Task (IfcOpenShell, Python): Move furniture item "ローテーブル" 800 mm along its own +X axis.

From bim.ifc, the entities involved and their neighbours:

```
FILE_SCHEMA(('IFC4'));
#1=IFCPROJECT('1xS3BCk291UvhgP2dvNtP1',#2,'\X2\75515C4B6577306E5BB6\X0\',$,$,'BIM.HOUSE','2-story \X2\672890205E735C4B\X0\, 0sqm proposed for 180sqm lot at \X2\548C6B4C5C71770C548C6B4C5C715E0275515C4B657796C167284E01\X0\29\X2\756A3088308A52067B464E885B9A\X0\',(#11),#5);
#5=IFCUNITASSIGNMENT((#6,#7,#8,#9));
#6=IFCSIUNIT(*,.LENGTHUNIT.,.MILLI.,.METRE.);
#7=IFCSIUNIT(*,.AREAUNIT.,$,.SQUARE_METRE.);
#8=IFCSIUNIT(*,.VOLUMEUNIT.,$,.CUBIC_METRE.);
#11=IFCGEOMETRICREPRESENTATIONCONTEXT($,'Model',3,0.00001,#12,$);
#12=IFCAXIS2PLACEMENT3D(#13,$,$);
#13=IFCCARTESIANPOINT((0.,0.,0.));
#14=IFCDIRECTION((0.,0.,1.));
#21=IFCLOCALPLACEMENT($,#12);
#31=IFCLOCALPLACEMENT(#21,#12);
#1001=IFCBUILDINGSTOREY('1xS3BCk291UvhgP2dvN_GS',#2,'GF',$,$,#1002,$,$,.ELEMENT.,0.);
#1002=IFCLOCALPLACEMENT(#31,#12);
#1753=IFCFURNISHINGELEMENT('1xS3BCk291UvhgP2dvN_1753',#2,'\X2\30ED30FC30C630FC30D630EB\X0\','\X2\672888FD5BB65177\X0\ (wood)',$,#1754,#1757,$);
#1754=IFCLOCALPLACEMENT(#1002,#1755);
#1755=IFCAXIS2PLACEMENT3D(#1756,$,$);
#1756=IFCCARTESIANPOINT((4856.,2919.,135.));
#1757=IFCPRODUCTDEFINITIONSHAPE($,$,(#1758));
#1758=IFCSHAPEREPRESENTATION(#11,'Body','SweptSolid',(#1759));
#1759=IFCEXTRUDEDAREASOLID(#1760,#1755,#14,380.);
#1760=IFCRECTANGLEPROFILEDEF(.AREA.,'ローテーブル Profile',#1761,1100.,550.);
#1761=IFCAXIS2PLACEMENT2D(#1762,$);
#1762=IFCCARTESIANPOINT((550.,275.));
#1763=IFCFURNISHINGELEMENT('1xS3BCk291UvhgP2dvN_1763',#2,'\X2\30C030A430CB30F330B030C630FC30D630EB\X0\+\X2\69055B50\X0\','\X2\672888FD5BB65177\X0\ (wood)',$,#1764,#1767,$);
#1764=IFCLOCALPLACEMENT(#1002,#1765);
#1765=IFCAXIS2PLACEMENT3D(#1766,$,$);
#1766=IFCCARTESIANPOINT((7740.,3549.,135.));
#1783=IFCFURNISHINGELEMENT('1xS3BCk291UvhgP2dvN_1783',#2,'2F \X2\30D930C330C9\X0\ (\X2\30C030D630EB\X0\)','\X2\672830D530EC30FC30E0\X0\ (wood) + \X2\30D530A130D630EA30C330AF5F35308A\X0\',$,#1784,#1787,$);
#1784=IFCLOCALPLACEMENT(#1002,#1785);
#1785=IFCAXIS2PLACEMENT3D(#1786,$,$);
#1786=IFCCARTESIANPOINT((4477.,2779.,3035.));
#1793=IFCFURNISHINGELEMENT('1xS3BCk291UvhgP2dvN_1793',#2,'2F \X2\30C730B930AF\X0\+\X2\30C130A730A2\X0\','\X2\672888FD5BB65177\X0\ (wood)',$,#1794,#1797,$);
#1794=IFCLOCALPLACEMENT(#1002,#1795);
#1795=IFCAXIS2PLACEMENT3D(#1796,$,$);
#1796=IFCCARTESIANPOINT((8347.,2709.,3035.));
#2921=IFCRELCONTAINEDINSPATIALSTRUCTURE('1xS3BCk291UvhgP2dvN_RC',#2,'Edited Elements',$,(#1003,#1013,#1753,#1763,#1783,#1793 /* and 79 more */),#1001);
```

```python
import ifcopenshell
import ifcopenshell.api.geometry
import ifcopenshell.util.placement
import ifcopenshell.util.unit

model = ifcopenshell.open("bim.ifc")
unit_scale = ifcopenshell.util.unit.calculate_unit_scale(model)

item = model.by_id(1753)
matrix = ifcopenshell.util.placement.get_local_placement(item.ObjectPlacement)
matrix[:3, 3] += matrix[:3, 0] * 0.8 / unit_scale
ifcopenshell.api.geometry.edit_object_placement(model, product=item, matrix=matrix, is_si=False)

print(ifcopenshell.util.placement.get_local_placement(item.ObjectPlacement).round(3) + 0.0)

model.write("bim_updated.ifc")
```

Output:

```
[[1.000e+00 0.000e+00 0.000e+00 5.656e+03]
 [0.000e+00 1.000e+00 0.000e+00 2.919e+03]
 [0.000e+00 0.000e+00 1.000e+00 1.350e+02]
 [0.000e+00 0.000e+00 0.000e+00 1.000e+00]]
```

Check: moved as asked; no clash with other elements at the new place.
